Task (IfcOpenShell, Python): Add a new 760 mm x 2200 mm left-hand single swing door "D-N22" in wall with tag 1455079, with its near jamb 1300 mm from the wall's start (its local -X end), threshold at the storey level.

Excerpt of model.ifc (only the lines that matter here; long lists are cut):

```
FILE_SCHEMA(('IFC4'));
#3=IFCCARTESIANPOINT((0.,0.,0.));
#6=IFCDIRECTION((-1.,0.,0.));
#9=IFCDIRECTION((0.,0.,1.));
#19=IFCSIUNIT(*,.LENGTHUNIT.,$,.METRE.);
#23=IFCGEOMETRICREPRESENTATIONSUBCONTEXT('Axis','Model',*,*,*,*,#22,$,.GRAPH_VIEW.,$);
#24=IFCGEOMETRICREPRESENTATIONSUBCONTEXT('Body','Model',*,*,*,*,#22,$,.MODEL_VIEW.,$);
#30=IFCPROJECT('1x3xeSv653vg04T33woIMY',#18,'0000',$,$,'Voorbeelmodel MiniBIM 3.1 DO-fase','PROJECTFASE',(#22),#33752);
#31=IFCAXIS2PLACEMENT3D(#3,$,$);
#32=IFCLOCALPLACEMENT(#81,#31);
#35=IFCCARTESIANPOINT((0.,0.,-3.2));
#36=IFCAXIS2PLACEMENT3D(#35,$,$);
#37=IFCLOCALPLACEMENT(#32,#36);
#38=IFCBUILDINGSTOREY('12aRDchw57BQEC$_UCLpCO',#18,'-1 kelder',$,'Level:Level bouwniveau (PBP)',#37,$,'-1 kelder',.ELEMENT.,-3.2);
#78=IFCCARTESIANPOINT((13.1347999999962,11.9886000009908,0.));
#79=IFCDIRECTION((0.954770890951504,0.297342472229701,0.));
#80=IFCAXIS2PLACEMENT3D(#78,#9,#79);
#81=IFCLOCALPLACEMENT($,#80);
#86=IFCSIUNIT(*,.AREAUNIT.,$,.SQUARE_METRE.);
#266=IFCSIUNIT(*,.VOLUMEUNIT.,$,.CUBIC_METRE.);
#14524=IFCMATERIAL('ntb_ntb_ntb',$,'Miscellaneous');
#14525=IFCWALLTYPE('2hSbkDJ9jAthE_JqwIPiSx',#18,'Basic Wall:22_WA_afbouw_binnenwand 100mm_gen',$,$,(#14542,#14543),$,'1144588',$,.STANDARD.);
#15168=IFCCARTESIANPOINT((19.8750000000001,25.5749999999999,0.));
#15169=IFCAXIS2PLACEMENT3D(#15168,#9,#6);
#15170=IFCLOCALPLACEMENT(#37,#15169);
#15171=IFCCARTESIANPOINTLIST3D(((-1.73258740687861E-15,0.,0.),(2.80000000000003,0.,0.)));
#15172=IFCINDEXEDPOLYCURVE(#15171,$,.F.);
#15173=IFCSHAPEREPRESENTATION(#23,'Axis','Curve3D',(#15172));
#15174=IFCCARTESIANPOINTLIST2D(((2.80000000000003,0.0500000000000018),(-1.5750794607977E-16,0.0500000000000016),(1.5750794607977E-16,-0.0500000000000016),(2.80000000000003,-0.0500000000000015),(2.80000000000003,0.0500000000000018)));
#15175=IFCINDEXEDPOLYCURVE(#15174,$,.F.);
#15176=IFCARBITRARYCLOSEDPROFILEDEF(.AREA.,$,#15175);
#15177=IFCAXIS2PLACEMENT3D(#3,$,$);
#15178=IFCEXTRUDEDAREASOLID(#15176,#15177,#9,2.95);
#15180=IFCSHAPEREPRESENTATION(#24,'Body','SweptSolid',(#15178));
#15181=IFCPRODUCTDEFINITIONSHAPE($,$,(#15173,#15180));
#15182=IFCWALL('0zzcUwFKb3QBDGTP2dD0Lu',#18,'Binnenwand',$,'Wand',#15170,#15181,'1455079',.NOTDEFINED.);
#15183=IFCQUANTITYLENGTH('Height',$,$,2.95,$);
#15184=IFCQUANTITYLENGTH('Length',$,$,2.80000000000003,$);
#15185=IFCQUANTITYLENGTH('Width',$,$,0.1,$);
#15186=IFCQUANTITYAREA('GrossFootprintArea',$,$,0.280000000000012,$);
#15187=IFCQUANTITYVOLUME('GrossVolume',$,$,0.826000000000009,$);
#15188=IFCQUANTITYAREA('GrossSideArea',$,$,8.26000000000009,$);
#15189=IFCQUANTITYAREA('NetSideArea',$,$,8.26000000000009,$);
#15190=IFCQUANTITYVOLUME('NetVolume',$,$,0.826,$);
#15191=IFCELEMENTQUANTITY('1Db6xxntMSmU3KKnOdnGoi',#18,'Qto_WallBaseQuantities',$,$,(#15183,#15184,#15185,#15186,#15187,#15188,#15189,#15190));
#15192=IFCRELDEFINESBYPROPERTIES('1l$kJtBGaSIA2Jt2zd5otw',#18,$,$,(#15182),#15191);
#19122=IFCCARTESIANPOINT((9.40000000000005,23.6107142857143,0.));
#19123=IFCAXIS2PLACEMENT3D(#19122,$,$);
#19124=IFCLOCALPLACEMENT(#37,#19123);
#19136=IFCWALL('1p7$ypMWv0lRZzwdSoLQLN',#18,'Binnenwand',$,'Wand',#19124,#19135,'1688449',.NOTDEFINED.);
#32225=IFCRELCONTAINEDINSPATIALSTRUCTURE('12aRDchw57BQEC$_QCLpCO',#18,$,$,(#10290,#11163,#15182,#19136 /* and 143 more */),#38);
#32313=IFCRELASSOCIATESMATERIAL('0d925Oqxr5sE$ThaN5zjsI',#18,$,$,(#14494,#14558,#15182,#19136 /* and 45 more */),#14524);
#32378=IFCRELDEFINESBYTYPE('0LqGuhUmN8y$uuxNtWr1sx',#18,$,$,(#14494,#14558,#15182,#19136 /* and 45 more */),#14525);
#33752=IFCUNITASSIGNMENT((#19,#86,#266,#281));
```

```python
import numpy as np
import ifcopenshell
import ifcopenshell.api.feature
import ifcopenshell.api.geometry
import ifcopenshell.api.pset
import ifcopenshell.api.root
import ifcopenshell.api.spatial
import ifcopenshell.geom
import ifcopenshell.util.element
import ifcopenshell.util.placement
import ifcopenshell.util.representation
import ifcopenshell.util.shape
import ifcopenshell.util.unit

model = ifcopenshell.open("model.ifc")
unit_scale = ifcopenshell.util.unit.calculate_unit_scale(model)
area_scale = ifcopenshell.util.unit.calculate_unit_scale(model, "AREAUNIT")
volume_scale = ifcopenshell.util.unit.calculate_unit_scale(model, "VOLUMEUNIT")
settings = ifcopenshell.geom.settings()


def volume(element):
    """Net volume in cubic metres, openings subtracted."""
    shape = ifcopenshell.geom.create_shape(settings, element)
    return ifcopenshell.util.shape.get_volume(shape.geometry)


wall = model.by_id(15182)
storey = ifcopenshell.util.element.get_container(wall, ifc_class="IfcBuildingStorey")
context = ifcopenshell.util.representation.get_context(model, "Model", "Body", "MODEL_VIEW")
before = volume(wall)

width, height, from_end, sill = 0.76, 2.2, 1.3, 0.0  # metres

# The wall runs along its own X axis, and the end named is its -X end.
wall_shape = ifcopenshell.geom.create_shape(settings, wall)
x, y, z = ifcopenshell.util.shape.get_vertices(wall_shape.geometry).T
start = x.min() + from_end
face, thickness = float(y.min()), float(y.max() - y.min())
wall_matrix = ifcopenshell.util.placement.get_local_placement(wall.ObjectPlacement)
level = ifcopenshell.util.placement.get_local_placement(storey.ObjectPlacement)[2, 3]


def in_wall(x, y):
    """Placement at x, y metres in the wall's axes, at sill height."""
    matrix = wall_matrix.copy()
    matrix[:, 3] = wall_matrix @ np.array([x / unit_scale, y / unit_scale, 0.0, 1.0])
    matrix[2, 3] = level + sill / unit_scale
    return matrix


# Opening: a box that overshoots both wall faces by 50 mm.
opening = ifcopenshell.api.root.create_entity(model, ifc_class="IfcOpeningElement", predefined_type="OPENING")
box = ifcopenshell.api.geometry.add_wall_representation(
    model, context=context, length=width, height=height, thickness=thickness + 0.1
)
ifcopenshell.api.geometry.assign_representation(model, product=opening, representation=box)
ifcopenshell.api.geometry.edit_object_placement(model, product=opening, matrix=in_wall(start, face - 0.05), is_si=False)
ifcopenshell.api.feature.add_feature(model, feature=opening, element=wall)

door = ifcopenshell.api.root.create_entity(model, ifc_class="IfcDoor", name="D-N22", predefined_type="DOOR")
door.OverallWidth, door.OverallHeight = width / unit_scale, height / unit_scale
door.OperationType = "SINGLE_SWING_LEFT"
body = ifcopenshell.api.geometry.add_door_representation(
    model,
    context=context,
    overall_width=door.OverallWidth,
    overall_height=door.OverallHeight,
    operation_type="SINGLE_SWING_LEFT",
    lining_properties={"LiningDepth": thickness / unit_scale, "ThresholdDepth": thickness / unit_scale},
)
ifcopenshell.api.geometry.assign_representation(model, product=door, representation=body)
ifcopenshell.api.spatial.assign_container(model, products=[door], relating_structure=storey)
ifcopenshell.api.feature.add_filling(model, opening=opening, element=door)

# The lining spans the wall, so the door starts at the wall face.
ifcopenshell.api.geometry.edit_object_placement(model, product=door, matrix=in_wall(start, face), is_si=False)

after = volume(wall)

# Update the wall's stored quantities.
qto = model.by_id(ifcopenshell.util.element.get_pset(wall, "Qto_WallBaseQuantities", should_inherit=False)["id"])
ifcopenshell.api.pset.edit_qto(model, qto=qto, properties={
    "NetSideArea": after / thickness / area_scale,
    "NetVolume": after / volume_scale,
})

print(f"wall volume {before:.3f} -> {after:.3f} m3")

model.write("model_edited.ifc")
```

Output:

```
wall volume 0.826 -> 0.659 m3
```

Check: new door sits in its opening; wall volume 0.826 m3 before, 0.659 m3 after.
